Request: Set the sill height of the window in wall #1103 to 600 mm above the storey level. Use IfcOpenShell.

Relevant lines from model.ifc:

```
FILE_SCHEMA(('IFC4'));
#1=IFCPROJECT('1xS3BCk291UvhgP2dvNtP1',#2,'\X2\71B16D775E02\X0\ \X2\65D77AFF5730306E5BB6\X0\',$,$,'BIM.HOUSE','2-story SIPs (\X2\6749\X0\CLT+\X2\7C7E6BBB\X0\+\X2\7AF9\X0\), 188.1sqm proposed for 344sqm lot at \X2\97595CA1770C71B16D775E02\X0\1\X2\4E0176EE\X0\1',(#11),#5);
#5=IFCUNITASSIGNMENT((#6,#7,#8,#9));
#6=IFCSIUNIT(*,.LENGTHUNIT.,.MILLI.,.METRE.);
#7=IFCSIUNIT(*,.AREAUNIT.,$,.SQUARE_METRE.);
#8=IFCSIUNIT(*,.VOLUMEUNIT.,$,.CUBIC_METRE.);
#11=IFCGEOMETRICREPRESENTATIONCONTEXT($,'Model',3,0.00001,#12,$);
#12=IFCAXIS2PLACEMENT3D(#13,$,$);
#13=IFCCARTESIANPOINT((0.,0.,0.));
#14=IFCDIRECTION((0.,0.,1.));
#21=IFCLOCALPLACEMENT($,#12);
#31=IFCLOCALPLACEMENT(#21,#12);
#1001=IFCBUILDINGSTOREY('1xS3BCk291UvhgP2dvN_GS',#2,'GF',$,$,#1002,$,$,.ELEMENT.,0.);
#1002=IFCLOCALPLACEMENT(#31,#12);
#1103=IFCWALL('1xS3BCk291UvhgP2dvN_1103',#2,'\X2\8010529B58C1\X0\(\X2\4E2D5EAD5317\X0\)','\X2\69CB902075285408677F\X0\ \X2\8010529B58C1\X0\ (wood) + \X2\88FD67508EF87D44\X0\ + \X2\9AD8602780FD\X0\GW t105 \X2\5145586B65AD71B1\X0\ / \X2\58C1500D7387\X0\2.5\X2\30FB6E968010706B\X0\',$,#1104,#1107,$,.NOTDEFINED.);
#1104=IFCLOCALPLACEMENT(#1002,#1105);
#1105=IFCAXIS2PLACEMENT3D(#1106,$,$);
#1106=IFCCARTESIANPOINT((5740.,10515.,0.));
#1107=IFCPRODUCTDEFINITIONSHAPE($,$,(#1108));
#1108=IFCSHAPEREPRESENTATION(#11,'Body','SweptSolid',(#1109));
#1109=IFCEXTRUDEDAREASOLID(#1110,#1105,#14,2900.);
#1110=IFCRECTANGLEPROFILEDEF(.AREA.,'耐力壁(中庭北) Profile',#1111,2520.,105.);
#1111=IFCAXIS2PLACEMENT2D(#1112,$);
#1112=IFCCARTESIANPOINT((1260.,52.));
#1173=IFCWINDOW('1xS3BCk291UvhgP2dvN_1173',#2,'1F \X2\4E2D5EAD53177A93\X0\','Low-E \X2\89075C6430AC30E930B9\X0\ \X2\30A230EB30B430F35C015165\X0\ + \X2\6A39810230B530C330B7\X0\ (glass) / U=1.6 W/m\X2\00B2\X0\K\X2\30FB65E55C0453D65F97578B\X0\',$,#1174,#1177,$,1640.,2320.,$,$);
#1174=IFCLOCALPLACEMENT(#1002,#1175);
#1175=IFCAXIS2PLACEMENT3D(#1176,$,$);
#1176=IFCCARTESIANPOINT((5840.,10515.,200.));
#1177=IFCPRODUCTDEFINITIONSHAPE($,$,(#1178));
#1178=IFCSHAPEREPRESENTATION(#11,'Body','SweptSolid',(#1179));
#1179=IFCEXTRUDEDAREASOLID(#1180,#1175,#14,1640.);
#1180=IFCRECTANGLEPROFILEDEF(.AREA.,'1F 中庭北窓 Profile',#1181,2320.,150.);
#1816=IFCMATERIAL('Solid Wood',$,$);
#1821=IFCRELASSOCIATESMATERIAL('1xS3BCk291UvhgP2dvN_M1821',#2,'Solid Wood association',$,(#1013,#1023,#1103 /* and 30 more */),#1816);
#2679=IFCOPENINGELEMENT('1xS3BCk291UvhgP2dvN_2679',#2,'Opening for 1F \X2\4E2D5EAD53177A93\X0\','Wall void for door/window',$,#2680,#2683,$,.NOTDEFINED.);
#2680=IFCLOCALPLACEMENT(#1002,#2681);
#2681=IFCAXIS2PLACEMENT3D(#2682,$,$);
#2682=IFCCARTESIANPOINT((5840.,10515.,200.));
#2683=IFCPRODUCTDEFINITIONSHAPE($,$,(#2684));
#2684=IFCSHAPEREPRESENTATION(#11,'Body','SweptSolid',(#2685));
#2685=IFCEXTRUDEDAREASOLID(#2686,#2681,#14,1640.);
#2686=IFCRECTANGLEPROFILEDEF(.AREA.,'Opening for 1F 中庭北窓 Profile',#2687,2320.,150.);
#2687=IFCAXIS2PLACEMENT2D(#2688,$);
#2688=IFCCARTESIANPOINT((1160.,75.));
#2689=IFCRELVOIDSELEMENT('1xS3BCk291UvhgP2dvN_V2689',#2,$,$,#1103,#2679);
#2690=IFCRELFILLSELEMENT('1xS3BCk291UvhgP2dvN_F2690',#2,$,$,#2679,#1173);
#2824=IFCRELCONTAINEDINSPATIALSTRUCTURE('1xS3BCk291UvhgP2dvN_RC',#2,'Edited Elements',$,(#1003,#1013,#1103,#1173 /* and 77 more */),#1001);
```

```python
import numpy as np
import ifcopenshell
import ifcopenshell.api.geometry
import ifcopenshell.geom
import ifcopenshell.util.element
import ifcopenshell.util.placement
import ifcopenshell.util.shape
import ifcopenshell.util.unit

model = ifcopenshell.open("model.ifc")
unit_scale = ifcopenshell.util.unit.calculate_unit_scale(model)

window = model.by_guid("1xS3BCk291UvhgP2dvN_1173")
opening = window.FillsVoids[0].RelatingOpeningElement
storey = ifcopenshell.util.element.get_container(window, ifc_class="IfcBuildingStorey")
level = ifcopenshell.util.placement.get_local_placement(storey.ObjectPlacement)[2, 3]

# The opening's origin need not be at the sill, so measure its lowest point.
shape = ifcopenshell.geom.create_shape(ifcopenshell.geom.settings(), opening)
bottom = ifcopenshell.util.shape.get_shape_bottom_elevation(shape, shape.geometry) / unit_scale
dz = level + 600.0 - bottom

shift = np.array([0.0, 0.0, dz])
# The window is not placed relative to its opening, so move both.
for product in (opening, window):
    matrix = ifcopenshell.util.placement.get_local_placement(product.ObjectPlacement)
    matrix[:3, 3] += shift
    ifcopenshell.api.geometry.edit_object_placement(model, product=product, matrix=matrix, is_si=False)

print(f"moved by {dz * unit_scale:+.3f} m")

model.write("model_edited.ifc")
```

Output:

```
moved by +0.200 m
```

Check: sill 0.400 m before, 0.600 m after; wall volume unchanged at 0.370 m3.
